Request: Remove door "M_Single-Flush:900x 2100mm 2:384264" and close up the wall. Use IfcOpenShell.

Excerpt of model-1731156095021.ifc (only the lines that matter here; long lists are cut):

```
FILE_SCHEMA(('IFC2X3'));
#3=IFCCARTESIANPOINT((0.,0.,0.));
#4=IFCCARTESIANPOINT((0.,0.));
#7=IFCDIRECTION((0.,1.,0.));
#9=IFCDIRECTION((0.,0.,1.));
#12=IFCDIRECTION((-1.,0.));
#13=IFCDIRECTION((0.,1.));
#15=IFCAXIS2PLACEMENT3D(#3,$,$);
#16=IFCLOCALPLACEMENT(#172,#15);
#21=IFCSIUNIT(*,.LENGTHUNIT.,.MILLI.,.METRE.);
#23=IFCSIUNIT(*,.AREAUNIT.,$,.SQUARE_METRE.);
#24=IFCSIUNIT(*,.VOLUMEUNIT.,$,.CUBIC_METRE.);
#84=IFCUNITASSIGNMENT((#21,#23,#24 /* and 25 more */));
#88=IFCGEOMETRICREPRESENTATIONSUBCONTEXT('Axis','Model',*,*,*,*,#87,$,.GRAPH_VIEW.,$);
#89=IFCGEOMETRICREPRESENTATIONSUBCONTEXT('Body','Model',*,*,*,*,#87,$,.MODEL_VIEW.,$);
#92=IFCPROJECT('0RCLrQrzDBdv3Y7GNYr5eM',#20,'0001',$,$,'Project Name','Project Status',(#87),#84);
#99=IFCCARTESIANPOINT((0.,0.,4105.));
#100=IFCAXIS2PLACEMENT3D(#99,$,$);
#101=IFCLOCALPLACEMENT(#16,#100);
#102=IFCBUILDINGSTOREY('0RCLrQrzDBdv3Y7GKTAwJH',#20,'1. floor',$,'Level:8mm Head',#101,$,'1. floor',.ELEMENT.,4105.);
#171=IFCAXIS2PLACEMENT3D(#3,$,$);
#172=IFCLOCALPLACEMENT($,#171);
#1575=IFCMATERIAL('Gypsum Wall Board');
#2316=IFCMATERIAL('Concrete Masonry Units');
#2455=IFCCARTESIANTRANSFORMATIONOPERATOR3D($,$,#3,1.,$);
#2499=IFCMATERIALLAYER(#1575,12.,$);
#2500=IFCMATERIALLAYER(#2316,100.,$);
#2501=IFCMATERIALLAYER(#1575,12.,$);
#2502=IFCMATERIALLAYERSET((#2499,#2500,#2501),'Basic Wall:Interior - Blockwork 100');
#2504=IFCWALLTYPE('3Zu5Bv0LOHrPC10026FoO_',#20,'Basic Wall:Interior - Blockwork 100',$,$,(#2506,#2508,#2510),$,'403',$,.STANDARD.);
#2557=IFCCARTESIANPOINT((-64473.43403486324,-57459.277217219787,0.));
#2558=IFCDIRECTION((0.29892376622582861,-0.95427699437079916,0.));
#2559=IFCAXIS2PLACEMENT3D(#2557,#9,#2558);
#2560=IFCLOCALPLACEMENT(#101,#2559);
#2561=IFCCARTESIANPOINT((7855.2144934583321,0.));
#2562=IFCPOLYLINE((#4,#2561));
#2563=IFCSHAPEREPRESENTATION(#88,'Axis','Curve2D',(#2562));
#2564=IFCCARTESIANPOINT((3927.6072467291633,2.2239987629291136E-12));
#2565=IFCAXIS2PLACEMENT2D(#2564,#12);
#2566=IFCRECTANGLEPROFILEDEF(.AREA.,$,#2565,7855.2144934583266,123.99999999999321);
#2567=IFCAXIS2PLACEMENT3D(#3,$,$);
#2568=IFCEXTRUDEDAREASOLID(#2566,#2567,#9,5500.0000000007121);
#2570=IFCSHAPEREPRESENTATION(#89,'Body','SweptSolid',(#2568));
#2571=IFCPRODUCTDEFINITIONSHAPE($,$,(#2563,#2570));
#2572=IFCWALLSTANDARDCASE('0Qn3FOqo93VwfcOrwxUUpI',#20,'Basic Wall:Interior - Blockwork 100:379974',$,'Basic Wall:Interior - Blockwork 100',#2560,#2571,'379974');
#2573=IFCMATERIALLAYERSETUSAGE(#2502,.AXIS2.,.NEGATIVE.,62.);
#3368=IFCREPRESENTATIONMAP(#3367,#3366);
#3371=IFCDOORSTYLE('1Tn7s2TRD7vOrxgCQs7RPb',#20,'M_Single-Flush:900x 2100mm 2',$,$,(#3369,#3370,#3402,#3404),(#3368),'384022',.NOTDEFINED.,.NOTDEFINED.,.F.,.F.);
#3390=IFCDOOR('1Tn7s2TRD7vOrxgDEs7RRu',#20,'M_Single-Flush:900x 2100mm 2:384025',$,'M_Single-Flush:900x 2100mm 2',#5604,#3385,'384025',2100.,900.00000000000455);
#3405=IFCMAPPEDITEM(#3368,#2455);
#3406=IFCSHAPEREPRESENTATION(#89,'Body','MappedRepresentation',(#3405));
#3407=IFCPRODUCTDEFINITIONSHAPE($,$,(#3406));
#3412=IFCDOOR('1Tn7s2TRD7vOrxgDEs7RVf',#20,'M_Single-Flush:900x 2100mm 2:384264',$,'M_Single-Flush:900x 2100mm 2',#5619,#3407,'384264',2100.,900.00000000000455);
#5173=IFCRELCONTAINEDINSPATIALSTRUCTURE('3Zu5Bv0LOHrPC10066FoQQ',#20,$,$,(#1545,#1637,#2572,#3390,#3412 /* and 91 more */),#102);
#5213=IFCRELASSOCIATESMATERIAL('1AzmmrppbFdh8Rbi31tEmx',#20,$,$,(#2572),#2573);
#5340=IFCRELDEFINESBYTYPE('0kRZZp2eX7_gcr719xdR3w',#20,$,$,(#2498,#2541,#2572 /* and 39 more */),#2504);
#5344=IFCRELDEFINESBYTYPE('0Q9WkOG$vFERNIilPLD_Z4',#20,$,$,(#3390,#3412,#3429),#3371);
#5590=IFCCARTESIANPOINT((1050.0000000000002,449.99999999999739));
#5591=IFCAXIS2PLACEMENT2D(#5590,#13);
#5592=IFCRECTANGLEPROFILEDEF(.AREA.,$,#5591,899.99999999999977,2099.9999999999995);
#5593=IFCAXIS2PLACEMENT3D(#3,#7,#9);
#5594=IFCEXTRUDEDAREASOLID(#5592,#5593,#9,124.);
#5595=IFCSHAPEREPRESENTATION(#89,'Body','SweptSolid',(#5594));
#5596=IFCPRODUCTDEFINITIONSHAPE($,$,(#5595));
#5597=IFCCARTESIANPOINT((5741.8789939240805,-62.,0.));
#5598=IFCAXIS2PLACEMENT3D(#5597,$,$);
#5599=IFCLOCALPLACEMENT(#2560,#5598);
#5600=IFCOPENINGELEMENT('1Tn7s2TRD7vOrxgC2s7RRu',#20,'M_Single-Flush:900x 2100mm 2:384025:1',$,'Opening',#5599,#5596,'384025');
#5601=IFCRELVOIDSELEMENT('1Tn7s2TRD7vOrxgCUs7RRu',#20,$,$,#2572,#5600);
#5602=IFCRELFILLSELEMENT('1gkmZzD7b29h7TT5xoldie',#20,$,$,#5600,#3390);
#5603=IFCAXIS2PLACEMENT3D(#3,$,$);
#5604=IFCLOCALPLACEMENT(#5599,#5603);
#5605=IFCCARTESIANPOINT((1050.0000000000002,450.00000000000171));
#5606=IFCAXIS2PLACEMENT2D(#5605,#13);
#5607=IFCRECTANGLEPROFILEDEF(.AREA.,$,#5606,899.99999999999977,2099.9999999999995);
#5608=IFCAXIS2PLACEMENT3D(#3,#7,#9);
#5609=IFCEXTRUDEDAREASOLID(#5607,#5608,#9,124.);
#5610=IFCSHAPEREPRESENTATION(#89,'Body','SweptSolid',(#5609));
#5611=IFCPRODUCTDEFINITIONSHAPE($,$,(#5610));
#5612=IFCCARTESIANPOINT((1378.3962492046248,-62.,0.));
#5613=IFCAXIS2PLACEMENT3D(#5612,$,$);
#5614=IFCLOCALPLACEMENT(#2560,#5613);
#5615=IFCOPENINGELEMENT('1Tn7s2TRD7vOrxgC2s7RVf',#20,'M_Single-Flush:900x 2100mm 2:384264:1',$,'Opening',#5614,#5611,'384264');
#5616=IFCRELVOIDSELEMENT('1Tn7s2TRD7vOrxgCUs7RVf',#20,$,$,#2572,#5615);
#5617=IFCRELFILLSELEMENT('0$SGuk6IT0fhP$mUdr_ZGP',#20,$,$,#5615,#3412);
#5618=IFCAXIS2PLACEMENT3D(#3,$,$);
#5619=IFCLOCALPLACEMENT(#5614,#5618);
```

```python
import ifcopenshell
import ifcopenshell.api.feature
import ifcopenshell.api.root
import ifcopenshell.geom
import ifcopenshell.util.shape

model = ifcopenshell.open("model-1731156095021.ifc")
settings = ifcopenshell.geom.settings()


def volume(element):
    """Net volume in cubic metres, openings subtracted."""
    shape = ifcopenshell.geom.create_shape(settings, element)
    return ifcopenshell.util.shape.get_volume(shape.geometry)


door = model.by_guid("1Tn7s2TRD7vOrxgDEs7RVf")
opening = door.FillsVoids[0].RelatingOpeningElement
wall = opening.VoidsElements[0].RelatingBuildingElement
before = volume(wall)

ifcopenshell.api.root.remove_product(model, product=door)
ifcopenshell.api.feature.remove_feature(model, feature=opening)

after = volume(wall)

print(f"wall volume {before:.3f} -> {after:.3f} m3")

model.write("model-1731156095021_edited.ifc")
```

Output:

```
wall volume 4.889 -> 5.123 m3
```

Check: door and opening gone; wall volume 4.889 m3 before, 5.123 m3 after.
